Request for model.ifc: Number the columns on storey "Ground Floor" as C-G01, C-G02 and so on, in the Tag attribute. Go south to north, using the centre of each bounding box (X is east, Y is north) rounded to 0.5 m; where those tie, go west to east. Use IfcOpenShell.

First a look at what the model holds.

```python
import ifcopenshell
import ifcopenshell.util.element
import ifcopenshell.util.placement

model = ifcopenshell.open("model.ifc")
print(model.schema)
storey = next(s for s in model.by_type("IfcBuildingStorey") if s.Name == "Ground Floor")
columns = [e for e in ifcopenshell.util.element.get_decomposition(storey) if e.is_a("IfcColumn")]
for e in sorted(columns, key=lambda e: e.id()):
    origin = ifcopenshell.util.placement.get_local_placement(e.ObjectPlacement)[:3, 3]
    print(e.id(), e.Tag, e.Name, origin.round(2) + 0.0, sep=" | ")
```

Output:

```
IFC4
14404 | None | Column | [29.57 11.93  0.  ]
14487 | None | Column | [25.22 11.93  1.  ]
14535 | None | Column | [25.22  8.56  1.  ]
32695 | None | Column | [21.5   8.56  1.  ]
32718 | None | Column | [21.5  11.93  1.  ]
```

```python
import ifcopenshell
import ifcopenshell.geom
import ifcopenshell.util.element
import ifcopenshell.util.shape

model = ifcopenshell.open("model.ifc")
settings = ifcopenshell.geom.settings()
settings.set("use-world-coords", True)


def centre(element):
    shape = ifcopenshell.geom.create_shape(settings, element)
    return ifcopenshell.util.shape.get_bbox_centroid(shape.geometry)


storey = next(s for s in model.by_type("IfcBuildingStorey") if s.Name == "Ground Floor")
columns = [e for e in ifcopenshell.util.element.get_decomposition(storey) if e.is_a("IfcColumn")]

# Insertion points can sit at a corner or the storey origin, so sort by the geometry (in metres).
centres = {e: centre(e) for e in columns}
columns.sort(key=lambda e: (round(centres[e][1] / 0.5), centres[e][0]))

for i, e in enumerate(columns, start=1):
    number = f"C-G{i:02d}"
    e.Tag = number
    print(e.id(), number)

model.write("model_edited.ifc")
```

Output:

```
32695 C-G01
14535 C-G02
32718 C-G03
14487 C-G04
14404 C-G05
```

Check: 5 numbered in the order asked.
